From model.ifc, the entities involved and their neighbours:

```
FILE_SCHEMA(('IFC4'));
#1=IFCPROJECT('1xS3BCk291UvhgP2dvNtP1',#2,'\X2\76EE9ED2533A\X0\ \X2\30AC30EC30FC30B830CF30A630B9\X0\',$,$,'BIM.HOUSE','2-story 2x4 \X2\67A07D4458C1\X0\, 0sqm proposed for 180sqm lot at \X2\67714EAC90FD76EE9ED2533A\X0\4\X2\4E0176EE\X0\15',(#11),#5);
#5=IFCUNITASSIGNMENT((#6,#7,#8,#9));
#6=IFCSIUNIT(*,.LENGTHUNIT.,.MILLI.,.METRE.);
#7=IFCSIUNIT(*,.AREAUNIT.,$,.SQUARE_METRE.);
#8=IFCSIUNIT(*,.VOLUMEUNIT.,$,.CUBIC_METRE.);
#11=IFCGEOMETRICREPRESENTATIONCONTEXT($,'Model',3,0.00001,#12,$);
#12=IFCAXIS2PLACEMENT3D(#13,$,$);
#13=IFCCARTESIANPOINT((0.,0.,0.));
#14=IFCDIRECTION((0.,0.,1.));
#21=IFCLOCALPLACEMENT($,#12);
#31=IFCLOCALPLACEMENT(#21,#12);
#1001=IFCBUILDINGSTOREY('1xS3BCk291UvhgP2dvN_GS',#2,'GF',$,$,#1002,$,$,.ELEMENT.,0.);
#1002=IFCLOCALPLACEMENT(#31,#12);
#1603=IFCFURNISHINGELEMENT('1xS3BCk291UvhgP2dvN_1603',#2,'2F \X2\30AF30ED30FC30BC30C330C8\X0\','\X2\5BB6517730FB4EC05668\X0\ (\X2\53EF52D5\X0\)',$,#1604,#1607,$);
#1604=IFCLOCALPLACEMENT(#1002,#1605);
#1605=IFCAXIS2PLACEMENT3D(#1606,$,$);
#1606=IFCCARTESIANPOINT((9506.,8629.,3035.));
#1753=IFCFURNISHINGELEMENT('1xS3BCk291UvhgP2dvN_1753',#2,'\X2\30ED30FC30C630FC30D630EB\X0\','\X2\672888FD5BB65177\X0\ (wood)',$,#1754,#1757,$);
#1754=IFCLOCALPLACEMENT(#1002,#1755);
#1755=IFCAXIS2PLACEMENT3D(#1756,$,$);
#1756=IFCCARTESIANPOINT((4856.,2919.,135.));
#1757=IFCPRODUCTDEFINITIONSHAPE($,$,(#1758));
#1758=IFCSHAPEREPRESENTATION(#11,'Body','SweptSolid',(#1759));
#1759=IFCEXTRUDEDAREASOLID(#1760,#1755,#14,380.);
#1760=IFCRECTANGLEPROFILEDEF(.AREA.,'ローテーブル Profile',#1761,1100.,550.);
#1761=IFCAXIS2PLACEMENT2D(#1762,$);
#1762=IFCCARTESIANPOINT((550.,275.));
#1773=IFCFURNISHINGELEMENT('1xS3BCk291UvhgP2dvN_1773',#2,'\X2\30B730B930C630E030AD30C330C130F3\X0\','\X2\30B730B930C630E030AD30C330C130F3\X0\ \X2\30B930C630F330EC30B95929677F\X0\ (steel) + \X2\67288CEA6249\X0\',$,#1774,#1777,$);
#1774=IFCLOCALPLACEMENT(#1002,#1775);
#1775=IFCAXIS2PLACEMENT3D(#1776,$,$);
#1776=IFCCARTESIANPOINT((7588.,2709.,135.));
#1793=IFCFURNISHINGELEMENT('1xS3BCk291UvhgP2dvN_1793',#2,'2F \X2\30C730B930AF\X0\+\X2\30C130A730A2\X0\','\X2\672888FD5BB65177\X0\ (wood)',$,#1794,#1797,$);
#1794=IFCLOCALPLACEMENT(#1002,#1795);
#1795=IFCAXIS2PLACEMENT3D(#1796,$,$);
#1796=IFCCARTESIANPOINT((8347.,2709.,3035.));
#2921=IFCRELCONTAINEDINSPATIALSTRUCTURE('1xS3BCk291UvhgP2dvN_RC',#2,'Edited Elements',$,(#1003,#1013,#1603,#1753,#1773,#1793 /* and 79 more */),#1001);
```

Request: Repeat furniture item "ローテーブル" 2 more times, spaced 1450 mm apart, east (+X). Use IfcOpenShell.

```python
import numpy as np
import ifcopenshell
import ifcopenshell.api.geometry
import ifcopenshell.api.root
import ifcopenshell.util.element
import ifcopenshell.util.placement
import ifcopenshell.util.unit

model = ifcopenshell.open("model.ifc")
unit_scale = ifcopenshell.util.unit.calculate_unit_scale(model)


def reuse_history(source, copy):
    """copy_class also copies each property set's owner history, people and application; keep the originals."""
    for rel in copy.IsDefinedBy:
        if rel.is_a("IfcRelDefinesByProperties") and (history := rel.RelatingPropertyDefinition.OwnerHistory):
            rel.RelatingPropertyDefinition.OwnerHistory = source.OwnerHistory
            ifcopenshell.util.element.remove_deep2(model, history)


source = model.by_guid("1xS3BCk291UvhgP2dvN_1753")
base = ifcopenshell.util.placement.get_local_placement(source.ObjectPlacement)
step = np.array([1.0, 0.0, 0.0]) * 1.45 / unit_scale

for i in range(1, 3):
    copy = ifcopenshell.api.root.copy_class(model, product=source)
    copy.Representation = ifcopenshell.util.element.copy_deep(
        model, source.Representation, exclude=["IfcGeometricRepresentationContext", "IfcRepresentationMap"]
    )
    reuse_history(source, copy)
    matrix = base.copy()
    matrix[:3, 3] += i * step
    print("added at", matrix[:3, 3].round(3) + 0.0)
    ifcopenshell.api.geometry.edit_object_placement(model, product=copy, matrix=matrix, is_si=False)

model.write("model_rev.ifc")
```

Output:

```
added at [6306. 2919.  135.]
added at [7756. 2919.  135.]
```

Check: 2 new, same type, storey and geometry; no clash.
